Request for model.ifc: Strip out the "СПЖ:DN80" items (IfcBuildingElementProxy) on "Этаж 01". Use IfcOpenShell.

First a look at what the model holds.

```python
import ifcopenshell
import ifcopenshell.util.element

model = ifcopenshell.open("model.ifc")
print(model.schema)
storey = next(s for s in model.by_type("IfcBuildingStorey") if s.Name == "Этаж 01")
proxies = [e for e in ifcopenshell.util.element.get_decomposition(storey) if e.is_a("IfcBuildingElementProxy")]
seen = {}
for e in proxies:
    element_type = ifcopenshell.util.element.get_type(e)
    name = element_type.Name if element_type not in (None, e) else None
    seen[name] = seen.get(name, 0) + 1
for name, count in sorted(seen.items(), key=str):
    print(count, "x", name)
```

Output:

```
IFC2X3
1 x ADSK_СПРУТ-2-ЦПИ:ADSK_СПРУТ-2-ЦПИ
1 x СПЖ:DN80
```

```python
import ifcopenshell
import ifcopenshell.api.root
import ifcopenshell.util.element

model = ifcopenshell.open("model.ifc")

storey = next(s for s in model.by_type("IfcBuildingStorey") if s.Name == "Этаж 01")
proxies = [e for e in ifcopenshell.util.element.get_decomposition(storey) if e.is_a("IfcBuildingElementProxy")]
targets = [e for e in proxies if (t := ifcopenshell.util.element.get_type(e)) not in (None, e) and t.Name == "СПЖ:DN80"]

for e in targets:
    ifcopenshell.api.root.remove_product(model, product=e)
print(len(targets), "removed")

model.write("model_edited.ifc")
```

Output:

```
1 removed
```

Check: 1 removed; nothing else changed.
